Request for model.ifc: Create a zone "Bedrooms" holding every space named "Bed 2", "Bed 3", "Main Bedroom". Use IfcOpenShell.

First a look at what the model holds.

```python
import ifcopenshell

model = ifcopenshell.open("model.ifc")
print(model.schema)
seen = {}
for space in model.by_type("IfcSpace"):
    seen[space.LongName] = seen.get(space.LongName, 0) + 1
for name, count in sorted(seen.items(), key=str):
    print(count, "x", name)
print("zones:", [z.Name for z in model.by_type("IfcZone")][:20])
```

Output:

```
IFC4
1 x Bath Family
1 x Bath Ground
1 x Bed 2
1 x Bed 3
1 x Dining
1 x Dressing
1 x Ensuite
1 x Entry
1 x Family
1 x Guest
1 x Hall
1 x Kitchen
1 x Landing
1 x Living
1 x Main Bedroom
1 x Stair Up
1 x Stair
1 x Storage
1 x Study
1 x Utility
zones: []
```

```python
import ifcopenshell
import ifcopenshell.api.group
import ifcopenshell.api.root

model = ifcopenshell.open("model.ifc")

names = {"Bed 2", "Bed 3", "Main Bedroom"}
spaces = [s for s in model.by_type("IfcSpace") if s.LongName in names]

zone = ifcopenshell.api.root.create_entity(model, ifc_class="IfcZone", name="Bedrooms")
ifcopenshell.api.group.assign_group(model, products=spaces, group=zone)
print(len(spaces), "spaces in", zone.Name)

model.write("model_updated.ifc")
```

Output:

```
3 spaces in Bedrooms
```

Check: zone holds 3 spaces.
